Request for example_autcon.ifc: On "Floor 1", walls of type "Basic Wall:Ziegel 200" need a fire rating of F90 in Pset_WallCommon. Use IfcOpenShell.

First a look at what the model holds.

```python
import ifcopenshell
import ifcopenshell.util.element

model = ifcopenshell.open("example_autcon.ifc")
print(model.schema)
storey = next(s for s in model.by_type("IfcBuildingStorey") if s.Name == "Floor 1")
walls = [e for e in ifcopenshell.util.element.get_decomposition(storey) if e.is_a("IfcWall")]
seen = {}
for e in walls:
    element_type = ifcopenshell.util.element.get_type(e)
    key = (element_type.Name if element_type != e and element_type else None, ifcopenshell.util.element.get_pset(e, "Pset_WallCommon", "FireRating"))
    seen[key] = seen.get(key, 0) + 1
for (name, value), count in sorted(seen.items(), key=str):
    print(count, "x", name, "|", value)
```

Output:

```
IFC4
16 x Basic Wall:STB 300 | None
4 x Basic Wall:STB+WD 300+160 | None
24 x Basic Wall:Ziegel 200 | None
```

```python
import ifcopenshell
import ifcopenshell.api.pset
import ifcopenshell.util.element

model = ifcopenshell.open("example_autcon.ifc")

storey = next(s for s in model.by_type("IfcBuildingStorey") if s.Name == "Floor 1")
walls = [e for e in ifcopenshell.util.element.get_decomposition(storey) if e.is_a("IfcWall")]

count = 0
for e in walls:
    element_type = ifcopenshell.util.element.get_type(e)
    if element_type in (None, e) or element_type.Name != "Basic Wall:Ziegel 200":
        continue
    # add_pset returns the element's existing set when there is one.
    pset = ifcopenshell.api.pset.add_pset(model, product=e, name="Pset_WallCommon")
    ifcopenshell.api.pset.edit_pset(model, pset=pset, properties={"FireRating": "F90"})
    count += 1

print(count, "walls updated")

model.write("example_autcon_updated.ifc")
```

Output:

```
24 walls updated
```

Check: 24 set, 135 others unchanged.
